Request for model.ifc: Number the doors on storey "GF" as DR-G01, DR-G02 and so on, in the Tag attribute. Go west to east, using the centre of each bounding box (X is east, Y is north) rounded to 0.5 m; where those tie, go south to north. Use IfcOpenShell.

First a look at what the model holds.

```python
import ifcopenshell
import ifcopenshell.util.element
import ifcopenshell.util.placement

model = ifcopenshell.open("model.ifc")
print(model.schema)
storey = next(s for s in model.by_type("IfcBuildingStorey") if s.Name == "GF")
doors = [e for e in ifcopenshell.util.element.get_decomposition(storey) if e.is_a("IfcDoor")]
for e in sorted(doors, key=lambda e: e.id()):
    origin = ifcopenshell.util.placement.get_local_placement(e.ObjectPlacement)[:3, 3]
    print(e.id(), e.Tag, e.Name, origin.round(2) + 0.0, sep=" | ")
```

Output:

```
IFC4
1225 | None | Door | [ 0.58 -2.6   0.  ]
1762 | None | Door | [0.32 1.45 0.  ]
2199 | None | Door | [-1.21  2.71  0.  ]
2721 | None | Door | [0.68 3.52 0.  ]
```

```python
import ifcopenshell
import ifcopenshell.geom
import ifcopenshell.util.element
import ifcopenshell.util.shape

model = ifcopenshell.open("model.ifc")
settings = ifcopenshell.geom.settings()
settings.set("use-world-coords", True)


def centre(element):
    shape = ifcopenshell.geom.create_shape(settings, element)
    return ifcopenshell.util.shape.get_bbox_centroid(shape.geometry)


storey = next(s for s in model.by_type("IfcBuildingStorey") if s.Name == "GF")
doors = [e for e in ifcopenshell.util.element.get_decomposition(storey) if e.is_a("IfcDoor")]

# Insertion points can sit at a corner or the storey origin, so sort by the geometry (in metres).
centres = {e: centre(e) for e in doors}
doors.sort(key=lambda e: (round(centres[e][0] / 0.5), centres[e][1]))

for i, e in enumerate(doors, start=1):
    number = f"DR-G{i:02d}"
    e.Tag = number
    print(e.id(), number)

model.write("model-out.ifc")
```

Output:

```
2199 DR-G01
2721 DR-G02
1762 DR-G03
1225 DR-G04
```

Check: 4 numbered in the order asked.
